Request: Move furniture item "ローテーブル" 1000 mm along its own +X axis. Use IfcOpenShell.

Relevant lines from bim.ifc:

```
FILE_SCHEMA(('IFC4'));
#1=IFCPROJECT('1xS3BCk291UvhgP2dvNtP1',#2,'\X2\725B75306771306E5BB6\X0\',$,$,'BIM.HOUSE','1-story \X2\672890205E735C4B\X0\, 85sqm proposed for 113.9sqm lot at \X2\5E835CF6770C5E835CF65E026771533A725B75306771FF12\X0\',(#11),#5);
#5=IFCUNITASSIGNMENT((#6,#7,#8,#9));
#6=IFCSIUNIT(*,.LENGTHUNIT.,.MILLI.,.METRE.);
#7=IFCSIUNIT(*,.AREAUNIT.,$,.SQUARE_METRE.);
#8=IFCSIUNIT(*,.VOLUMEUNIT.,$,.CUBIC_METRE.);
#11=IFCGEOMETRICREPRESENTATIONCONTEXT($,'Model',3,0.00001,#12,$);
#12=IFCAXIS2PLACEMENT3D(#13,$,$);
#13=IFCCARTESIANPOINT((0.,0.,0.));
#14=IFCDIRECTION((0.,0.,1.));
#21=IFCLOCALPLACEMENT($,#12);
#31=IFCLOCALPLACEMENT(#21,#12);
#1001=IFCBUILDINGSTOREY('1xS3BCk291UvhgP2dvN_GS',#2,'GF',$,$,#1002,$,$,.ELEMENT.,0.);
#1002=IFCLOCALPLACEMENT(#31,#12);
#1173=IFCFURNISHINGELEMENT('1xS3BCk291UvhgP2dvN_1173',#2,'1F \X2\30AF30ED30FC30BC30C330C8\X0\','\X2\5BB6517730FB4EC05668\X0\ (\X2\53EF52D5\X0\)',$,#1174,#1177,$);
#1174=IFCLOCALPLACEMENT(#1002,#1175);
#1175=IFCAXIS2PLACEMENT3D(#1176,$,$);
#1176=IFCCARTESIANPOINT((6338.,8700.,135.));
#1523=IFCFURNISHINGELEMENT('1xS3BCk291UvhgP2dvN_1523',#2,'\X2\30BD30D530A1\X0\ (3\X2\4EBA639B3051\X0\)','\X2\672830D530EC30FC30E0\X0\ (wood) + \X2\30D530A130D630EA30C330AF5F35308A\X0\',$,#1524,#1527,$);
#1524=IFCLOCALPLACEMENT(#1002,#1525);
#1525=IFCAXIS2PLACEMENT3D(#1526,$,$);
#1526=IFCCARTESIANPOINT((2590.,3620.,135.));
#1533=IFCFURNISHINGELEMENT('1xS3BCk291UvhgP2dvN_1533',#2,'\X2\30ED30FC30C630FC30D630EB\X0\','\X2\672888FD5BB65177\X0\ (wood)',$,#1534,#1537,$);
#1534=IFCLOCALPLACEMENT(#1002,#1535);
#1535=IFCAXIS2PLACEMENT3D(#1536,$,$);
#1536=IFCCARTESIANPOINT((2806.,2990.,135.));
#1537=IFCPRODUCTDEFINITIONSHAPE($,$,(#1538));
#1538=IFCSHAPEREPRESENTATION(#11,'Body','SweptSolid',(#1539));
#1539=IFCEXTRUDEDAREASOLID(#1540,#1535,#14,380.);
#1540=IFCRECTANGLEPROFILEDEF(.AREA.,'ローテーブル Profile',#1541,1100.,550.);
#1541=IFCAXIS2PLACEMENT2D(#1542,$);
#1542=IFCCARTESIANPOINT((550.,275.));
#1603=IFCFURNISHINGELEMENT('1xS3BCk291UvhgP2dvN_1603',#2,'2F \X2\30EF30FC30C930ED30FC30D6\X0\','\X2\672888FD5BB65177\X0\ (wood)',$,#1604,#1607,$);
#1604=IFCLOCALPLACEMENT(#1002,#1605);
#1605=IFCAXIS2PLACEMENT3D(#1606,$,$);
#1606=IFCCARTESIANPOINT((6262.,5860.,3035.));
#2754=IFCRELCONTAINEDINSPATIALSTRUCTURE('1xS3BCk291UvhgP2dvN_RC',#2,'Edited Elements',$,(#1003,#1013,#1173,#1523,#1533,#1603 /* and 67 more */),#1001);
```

```python
import ifcopenshell
import ifcopenshell.api.geometry
import ifcopenshell.util.placement
import ifcopenshell.util.unit

model = ifcopenshell.open("bim.ifc")
unit_scale = ifcopenshell.util.unit.calculate_unit_scale(model)

item = model.by_guid("1xS3BCk291UvhgP2dvN_1533")
matrix = ifcopenshell.util.placement.get_local_placement(item.ObjectPlacement)
matrix[:3, 3] += matrix[:3, 0] * 1 / unit_scale
ifcopenshell.api.geometry.edit_object_placement(model, product=item, matrix=matrix, is_si=False)

print(ifcopenshell.util.placement.get_local_placement(item.ObjectPlacement).round(3) + 0.0)

model.write("bim_updated.ifc")
```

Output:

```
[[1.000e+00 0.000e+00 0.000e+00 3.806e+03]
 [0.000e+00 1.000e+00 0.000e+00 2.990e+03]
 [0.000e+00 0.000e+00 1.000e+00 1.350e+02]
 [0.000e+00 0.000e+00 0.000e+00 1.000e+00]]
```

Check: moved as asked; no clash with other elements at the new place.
